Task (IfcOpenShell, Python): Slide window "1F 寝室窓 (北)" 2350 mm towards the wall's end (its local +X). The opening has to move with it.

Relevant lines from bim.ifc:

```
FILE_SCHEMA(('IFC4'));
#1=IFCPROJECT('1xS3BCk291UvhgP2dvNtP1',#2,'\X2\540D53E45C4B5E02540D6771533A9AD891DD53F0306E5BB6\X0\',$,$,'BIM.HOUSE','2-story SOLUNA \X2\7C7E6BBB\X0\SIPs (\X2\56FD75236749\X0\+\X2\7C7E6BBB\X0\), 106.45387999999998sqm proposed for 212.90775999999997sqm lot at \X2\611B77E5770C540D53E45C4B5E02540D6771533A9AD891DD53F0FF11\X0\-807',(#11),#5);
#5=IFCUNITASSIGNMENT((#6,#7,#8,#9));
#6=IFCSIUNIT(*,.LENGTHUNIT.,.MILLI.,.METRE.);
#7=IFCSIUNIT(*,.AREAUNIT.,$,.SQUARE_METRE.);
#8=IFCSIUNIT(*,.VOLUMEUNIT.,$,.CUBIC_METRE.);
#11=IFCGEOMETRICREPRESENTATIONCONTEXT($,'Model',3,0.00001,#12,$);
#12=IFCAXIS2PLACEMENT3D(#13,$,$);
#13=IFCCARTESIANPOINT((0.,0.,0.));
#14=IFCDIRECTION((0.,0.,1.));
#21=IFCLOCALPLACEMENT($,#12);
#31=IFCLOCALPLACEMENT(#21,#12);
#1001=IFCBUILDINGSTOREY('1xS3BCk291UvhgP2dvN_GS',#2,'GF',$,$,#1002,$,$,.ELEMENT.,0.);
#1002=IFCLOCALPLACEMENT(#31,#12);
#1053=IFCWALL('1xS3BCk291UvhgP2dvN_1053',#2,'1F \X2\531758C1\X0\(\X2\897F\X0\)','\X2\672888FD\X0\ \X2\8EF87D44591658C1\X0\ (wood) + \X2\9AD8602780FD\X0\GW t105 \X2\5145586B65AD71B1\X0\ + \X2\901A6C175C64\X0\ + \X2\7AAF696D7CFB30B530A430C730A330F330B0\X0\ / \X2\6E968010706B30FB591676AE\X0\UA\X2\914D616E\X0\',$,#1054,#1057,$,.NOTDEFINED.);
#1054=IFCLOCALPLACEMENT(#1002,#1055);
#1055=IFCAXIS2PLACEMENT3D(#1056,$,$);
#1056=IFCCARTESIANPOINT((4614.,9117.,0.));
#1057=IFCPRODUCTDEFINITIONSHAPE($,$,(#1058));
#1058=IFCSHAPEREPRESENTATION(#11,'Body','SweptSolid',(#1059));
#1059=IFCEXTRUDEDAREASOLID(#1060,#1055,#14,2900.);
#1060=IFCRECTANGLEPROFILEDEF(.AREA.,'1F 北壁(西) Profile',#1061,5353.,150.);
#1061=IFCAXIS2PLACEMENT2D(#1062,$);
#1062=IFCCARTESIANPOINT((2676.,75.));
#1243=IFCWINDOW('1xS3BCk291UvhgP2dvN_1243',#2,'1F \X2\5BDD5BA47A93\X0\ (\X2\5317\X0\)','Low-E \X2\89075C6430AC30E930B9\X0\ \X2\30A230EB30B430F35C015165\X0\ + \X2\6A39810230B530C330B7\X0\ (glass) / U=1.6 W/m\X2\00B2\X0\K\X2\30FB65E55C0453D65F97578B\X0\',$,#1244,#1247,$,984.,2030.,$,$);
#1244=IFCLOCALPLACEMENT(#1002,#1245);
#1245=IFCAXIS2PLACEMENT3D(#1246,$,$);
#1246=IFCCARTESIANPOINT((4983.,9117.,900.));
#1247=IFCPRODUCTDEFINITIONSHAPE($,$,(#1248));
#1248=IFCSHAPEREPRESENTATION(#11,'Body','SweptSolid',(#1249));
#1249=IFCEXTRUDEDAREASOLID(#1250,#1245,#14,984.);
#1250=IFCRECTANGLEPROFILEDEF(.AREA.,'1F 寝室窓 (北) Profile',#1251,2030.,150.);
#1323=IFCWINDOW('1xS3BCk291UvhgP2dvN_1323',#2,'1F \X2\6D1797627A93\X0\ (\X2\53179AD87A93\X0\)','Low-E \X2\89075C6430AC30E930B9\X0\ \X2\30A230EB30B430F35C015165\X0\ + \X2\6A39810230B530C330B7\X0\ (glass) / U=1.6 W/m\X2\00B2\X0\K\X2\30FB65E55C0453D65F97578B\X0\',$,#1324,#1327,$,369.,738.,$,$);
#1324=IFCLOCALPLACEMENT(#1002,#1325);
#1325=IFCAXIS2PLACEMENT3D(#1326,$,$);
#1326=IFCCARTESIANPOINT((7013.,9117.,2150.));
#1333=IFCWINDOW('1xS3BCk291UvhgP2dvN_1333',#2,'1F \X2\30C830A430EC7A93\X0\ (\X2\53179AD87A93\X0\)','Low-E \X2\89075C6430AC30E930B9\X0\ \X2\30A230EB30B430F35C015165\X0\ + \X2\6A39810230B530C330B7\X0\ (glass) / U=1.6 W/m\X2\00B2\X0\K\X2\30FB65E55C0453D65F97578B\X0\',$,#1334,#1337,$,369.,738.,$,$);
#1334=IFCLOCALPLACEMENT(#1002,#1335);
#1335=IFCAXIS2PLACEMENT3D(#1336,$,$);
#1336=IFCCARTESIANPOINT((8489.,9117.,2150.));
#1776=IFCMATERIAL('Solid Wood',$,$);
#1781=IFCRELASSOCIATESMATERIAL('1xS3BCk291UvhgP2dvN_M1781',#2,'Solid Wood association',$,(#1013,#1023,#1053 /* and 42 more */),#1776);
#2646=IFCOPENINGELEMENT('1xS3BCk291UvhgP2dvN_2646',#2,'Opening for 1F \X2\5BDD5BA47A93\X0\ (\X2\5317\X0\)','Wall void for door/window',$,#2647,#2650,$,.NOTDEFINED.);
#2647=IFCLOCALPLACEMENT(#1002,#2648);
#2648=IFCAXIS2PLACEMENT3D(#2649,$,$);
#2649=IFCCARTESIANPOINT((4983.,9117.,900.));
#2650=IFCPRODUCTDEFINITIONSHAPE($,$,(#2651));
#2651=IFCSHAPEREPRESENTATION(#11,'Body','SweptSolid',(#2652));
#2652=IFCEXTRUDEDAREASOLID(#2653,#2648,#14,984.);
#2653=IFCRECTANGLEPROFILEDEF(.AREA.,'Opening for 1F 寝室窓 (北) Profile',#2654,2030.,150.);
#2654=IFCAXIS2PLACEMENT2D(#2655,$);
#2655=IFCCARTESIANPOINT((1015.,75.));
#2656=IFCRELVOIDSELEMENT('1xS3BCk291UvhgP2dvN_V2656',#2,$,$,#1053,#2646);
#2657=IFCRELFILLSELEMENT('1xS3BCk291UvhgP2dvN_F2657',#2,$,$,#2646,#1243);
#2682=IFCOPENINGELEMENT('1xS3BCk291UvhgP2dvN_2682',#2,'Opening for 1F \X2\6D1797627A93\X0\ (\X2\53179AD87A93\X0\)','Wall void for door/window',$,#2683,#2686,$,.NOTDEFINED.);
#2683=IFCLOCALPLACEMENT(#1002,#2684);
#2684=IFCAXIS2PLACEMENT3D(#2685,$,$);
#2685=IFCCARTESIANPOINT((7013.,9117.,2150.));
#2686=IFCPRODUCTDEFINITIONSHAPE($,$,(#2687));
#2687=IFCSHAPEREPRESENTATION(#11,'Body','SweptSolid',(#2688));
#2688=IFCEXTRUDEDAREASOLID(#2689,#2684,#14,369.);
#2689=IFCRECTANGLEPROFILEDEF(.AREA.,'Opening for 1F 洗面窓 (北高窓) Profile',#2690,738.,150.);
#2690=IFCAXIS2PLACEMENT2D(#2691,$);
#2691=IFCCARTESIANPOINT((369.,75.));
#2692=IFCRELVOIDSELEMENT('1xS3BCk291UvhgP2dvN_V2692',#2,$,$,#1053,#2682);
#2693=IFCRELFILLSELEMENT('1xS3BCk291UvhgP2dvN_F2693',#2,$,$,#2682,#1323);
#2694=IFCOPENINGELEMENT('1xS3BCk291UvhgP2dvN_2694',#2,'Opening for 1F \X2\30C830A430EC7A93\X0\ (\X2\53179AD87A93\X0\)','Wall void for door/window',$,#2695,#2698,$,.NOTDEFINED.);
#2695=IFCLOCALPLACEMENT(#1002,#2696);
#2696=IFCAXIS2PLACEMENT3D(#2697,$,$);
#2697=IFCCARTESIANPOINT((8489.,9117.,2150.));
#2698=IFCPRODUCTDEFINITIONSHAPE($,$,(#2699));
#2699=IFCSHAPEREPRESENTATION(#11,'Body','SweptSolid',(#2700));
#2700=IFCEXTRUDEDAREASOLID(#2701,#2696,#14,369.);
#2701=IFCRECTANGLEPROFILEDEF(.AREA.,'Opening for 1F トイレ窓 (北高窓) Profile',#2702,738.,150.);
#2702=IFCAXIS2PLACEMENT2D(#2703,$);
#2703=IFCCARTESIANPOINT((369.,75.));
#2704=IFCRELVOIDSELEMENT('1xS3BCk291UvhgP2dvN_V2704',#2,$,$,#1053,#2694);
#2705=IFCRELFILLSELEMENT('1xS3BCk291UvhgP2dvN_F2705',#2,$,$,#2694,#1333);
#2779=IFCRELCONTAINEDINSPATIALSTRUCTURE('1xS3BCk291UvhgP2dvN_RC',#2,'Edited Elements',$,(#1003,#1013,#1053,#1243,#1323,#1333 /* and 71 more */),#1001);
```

```python
import ifcopenshell
import ifcopenshell.api.geometry
import ifcopenshell.util.placement

model = ifcopenshell.open("bim.ifc")

window = model.by_guid("1xS3BCk291UvhgP2dvN_1243")
opening = window.FillsVoids[0].RelatingOpeningElement
wall = opening.VoidsElements[0].RelatingBuildingElement

wall_matrix = ifcopenshell.util.placement.get_local_placement(wall.ObjectPlacement)
shift = wall_matrix[:3, 0] * 2350.0
before = ifcopenshell.util.placement.get_local_placement(window.ObjectPlacement)[:3, 3].copy()

# The window is not placed relative to its opening, so move both.
for product in (opening, window):
    matrix = ifcopenshell.util.placement.get_local_placement(product.ObjectPlacement)
    matrix[:3, 3] += shift
    ifcopenshell.api.geometry.edit_object_placement(model, product=product, matrix=matrix, is_si=False)

after = ifcopenshell.util.placement.get_local_placement(window.ObjectPlacement)[:3, 3]
print("window moved by", (after - before).round(3) + 0.0)

model.write("bim_edited.ifc")
```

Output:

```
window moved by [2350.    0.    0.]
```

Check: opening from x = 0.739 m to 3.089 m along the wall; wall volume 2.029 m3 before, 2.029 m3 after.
